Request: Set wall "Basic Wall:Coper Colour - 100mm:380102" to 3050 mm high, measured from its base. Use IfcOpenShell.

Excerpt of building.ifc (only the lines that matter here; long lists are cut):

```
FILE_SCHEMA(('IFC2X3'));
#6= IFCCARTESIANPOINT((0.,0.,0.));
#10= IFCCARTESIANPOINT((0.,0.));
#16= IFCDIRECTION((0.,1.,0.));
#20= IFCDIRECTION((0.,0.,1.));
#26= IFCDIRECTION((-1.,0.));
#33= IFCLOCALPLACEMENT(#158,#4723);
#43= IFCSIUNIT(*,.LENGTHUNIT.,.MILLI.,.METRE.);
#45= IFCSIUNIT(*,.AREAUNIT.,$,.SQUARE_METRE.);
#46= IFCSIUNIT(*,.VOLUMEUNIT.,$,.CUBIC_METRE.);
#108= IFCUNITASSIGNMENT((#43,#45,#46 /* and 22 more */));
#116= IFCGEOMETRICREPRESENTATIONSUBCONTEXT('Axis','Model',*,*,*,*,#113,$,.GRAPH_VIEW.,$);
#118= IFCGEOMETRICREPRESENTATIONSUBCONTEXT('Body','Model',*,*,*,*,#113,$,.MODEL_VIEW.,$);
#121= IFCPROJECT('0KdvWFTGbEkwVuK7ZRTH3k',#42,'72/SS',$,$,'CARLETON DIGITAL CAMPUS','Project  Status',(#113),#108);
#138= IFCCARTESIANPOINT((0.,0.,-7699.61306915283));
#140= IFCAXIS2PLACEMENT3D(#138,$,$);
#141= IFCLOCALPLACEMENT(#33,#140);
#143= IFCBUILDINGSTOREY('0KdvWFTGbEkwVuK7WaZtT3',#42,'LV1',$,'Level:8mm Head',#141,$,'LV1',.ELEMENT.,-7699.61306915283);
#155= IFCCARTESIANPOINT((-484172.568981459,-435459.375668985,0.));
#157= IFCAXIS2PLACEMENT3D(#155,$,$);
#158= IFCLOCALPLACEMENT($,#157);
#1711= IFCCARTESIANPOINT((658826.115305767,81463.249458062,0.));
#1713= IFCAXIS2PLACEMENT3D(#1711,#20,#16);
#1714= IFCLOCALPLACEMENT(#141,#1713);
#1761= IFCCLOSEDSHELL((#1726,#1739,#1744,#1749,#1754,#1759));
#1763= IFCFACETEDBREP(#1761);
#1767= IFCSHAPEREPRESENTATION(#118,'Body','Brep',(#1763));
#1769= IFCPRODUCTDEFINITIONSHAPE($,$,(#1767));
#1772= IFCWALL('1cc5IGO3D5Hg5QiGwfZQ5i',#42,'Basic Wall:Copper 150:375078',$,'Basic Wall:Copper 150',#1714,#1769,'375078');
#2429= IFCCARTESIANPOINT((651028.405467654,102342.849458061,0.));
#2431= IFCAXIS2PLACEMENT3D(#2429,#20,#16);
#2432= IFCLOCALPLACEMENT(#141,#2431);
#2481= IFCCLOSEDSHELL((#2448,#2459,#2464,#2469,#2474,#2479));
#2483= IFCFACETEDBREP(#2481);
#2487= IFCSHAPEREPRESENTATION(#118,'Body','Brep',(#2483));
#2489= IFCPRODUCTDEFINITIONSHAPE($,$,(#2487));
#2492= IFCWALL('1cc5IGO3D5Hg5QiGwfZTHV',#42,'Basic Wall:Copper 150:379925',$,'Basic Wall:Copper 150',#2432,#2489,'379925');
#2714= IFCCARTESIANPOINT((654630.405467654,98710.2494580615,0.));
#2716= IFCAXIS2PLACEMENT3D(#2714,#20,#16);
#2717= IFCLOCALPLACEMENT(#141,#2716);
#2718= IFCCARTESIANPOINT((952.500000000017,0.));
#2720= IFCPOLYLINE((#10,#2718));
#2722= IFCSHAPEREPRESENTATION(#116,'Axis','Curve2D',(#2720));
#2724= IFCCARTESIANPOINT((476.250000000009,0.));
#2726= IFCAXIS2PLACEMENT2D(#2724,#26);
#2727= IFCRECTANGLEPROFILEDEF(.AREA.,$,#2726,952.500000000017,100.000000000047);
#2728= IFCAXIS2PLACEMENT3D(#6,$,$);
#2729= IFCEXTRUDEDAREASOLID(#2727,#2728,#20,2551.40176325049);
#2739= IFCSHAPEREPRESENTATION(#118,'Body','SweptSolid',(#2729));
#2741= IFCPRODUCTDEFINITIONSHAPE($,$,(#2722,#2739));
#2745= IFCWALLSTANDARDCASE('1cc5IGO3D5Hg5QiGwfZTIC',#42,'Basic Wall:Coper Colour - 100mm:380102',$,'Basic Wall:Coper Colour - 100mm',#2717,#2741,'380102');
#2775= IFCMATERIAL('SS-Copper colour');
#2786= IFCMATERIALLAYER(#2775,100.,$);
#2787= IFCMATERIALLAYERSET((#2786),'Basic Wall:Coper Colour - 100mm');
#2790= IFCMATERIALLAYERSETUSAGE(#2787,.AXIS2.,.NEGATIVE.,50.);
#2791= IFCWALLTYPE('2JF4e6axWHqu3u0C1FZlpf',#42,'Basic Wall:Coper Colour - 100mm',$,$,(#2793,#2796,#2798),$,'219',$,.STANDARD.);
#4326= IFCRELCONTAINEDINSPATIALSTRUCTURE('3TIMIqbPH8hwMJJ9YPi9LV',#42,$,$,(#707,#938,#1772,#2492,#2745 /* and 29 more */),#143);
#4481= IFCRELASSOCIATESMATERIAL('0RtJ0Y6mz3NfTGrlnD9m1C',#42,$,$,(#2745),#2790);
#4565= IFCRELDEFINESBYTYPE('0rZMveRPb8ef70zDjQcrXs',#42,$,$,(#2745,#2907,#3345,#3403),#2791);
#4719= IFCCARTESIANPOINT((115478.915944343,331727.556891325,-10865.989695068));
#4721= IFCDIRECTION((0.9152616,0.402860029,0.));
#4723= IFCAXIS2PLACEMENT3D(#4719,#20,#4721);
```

```python
import ifcopenshell
import ifcopenshell.geom
import ifcopenshell.util.representation
import ifcopenshell.util.shape
import ifcopenshell.util.unit

model = ifcopenshell.open("building.ifc")
unit_scale = ifcopenshell.util.unit.calculate_unit_scale(model)
settings = ifcopenshell.geom.settings()


def volume(element):
    """Net volume in cubic metres, openings subtracted."""
    shape = ifcopenshell.geom.create_shape(settings, element)
    return ifcopenshell.util.shape.get_volume(shape.geometry)


wall = model.by_guid("1cc5IGO3D5Hg5QiGwfZTIC")
before = volume(wall)

body = ifcopenshell.util.representation.get_representation(wall, "Model", "Body")
solid = body.Items[0]
old_height = solid.Depth
solid.Depth = 3.05 / unit_scale
after = volume(wall)

print(f"height {old_height:g} -> {solid.Depth:g}, volume {before:.3f} -> {after:.3f} m3")

model.write("building_updated.ifc")
```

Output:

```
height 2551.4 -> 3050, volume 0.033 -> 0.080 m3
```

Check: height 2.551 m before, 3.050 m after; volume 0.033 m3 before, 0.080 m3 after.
